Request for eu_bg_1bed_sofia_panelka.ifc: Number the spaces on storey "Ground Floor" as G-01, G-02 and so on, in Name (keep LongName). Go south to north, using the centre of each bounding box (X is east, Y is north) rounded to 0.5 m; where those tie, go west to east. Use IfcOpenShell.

First a look at what the model holds.

```python
import ifcopenshell
import ifcopenshell.util.element
import ifcopenshell.util.placement

model = ifcopenshell.open("eu_bg_1bed_sofia_panelka.ifc")
print(model.schema)
storey = next(s for s in model.by_type("IfcBuildingStorey") if s.Name == "Ground Floor")
spaces = [e for e in ifcopenshell.util.element.get_decomposition(storey) if e.is_a("IfcSpace")]
for e in sorted(spaces, key=lambda e: e.id()):
    origin = ifcopenshell.util.placement.get_local_placement(e.ObjectPlacement)[:3, 3]
    print(e.id(), e.Name, e.LongName, origin.round(2) + 0.0, sep=" | ")
```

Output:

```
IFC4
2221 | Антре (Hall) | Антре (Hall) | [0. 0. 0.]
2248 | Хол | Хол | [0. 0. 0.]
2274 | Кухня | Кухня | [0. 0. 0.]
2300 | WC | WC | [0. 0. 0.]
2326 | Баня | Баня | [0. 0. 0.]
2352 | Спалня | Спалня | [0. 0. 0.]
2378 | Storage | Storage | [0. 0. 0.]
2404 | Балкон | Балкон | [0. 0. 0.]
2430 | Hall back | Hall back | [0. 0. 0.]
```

```python
import ifcopenshell
import ifcopenshell.geom
import ifcopenshell.util.element
import ifcopenshell.util.shape

model = ifcopenshell.open("eu_bg_1bed_sofia_panelka.ifc")
settings = ifcopenshell.geom.settings()
settings.set("use-world-coords", True)


def centre(element):
    shape = ifcopenshell.geom.create_shape(settings, element)
    return ifcopenshell.util.shape.get_bbox_centroid(shape.geometry)


storey = next(s for s in model.by_type("IfcBuildingStorey") if s.Name == "Ground Floor")
spaces = [e for e in ifcopenshell.util.element.get_decomposition(storey) if e.is_a("IfcSpace")]

# Insertion points can sit at a corner or the storey origin, so sort by the geometry (in metres).
centres = {e: centre(e) for e in spaces}
spaces.sort(key=lambda e: (round(centres[e][1] / 0.5), centres[e][0]))

for i, e in enumerate(spaces, start=1):
    number = f"G-{i:02d}"
    e.Name = number
    print(e.id(), number)

model.write("eu_bg_1bed_sofia_panelka_rev.ifc")
```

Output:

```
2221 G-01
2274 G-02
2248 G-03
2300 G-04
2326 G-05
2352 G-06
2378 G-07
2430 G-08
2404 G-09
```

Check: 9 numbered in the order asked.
